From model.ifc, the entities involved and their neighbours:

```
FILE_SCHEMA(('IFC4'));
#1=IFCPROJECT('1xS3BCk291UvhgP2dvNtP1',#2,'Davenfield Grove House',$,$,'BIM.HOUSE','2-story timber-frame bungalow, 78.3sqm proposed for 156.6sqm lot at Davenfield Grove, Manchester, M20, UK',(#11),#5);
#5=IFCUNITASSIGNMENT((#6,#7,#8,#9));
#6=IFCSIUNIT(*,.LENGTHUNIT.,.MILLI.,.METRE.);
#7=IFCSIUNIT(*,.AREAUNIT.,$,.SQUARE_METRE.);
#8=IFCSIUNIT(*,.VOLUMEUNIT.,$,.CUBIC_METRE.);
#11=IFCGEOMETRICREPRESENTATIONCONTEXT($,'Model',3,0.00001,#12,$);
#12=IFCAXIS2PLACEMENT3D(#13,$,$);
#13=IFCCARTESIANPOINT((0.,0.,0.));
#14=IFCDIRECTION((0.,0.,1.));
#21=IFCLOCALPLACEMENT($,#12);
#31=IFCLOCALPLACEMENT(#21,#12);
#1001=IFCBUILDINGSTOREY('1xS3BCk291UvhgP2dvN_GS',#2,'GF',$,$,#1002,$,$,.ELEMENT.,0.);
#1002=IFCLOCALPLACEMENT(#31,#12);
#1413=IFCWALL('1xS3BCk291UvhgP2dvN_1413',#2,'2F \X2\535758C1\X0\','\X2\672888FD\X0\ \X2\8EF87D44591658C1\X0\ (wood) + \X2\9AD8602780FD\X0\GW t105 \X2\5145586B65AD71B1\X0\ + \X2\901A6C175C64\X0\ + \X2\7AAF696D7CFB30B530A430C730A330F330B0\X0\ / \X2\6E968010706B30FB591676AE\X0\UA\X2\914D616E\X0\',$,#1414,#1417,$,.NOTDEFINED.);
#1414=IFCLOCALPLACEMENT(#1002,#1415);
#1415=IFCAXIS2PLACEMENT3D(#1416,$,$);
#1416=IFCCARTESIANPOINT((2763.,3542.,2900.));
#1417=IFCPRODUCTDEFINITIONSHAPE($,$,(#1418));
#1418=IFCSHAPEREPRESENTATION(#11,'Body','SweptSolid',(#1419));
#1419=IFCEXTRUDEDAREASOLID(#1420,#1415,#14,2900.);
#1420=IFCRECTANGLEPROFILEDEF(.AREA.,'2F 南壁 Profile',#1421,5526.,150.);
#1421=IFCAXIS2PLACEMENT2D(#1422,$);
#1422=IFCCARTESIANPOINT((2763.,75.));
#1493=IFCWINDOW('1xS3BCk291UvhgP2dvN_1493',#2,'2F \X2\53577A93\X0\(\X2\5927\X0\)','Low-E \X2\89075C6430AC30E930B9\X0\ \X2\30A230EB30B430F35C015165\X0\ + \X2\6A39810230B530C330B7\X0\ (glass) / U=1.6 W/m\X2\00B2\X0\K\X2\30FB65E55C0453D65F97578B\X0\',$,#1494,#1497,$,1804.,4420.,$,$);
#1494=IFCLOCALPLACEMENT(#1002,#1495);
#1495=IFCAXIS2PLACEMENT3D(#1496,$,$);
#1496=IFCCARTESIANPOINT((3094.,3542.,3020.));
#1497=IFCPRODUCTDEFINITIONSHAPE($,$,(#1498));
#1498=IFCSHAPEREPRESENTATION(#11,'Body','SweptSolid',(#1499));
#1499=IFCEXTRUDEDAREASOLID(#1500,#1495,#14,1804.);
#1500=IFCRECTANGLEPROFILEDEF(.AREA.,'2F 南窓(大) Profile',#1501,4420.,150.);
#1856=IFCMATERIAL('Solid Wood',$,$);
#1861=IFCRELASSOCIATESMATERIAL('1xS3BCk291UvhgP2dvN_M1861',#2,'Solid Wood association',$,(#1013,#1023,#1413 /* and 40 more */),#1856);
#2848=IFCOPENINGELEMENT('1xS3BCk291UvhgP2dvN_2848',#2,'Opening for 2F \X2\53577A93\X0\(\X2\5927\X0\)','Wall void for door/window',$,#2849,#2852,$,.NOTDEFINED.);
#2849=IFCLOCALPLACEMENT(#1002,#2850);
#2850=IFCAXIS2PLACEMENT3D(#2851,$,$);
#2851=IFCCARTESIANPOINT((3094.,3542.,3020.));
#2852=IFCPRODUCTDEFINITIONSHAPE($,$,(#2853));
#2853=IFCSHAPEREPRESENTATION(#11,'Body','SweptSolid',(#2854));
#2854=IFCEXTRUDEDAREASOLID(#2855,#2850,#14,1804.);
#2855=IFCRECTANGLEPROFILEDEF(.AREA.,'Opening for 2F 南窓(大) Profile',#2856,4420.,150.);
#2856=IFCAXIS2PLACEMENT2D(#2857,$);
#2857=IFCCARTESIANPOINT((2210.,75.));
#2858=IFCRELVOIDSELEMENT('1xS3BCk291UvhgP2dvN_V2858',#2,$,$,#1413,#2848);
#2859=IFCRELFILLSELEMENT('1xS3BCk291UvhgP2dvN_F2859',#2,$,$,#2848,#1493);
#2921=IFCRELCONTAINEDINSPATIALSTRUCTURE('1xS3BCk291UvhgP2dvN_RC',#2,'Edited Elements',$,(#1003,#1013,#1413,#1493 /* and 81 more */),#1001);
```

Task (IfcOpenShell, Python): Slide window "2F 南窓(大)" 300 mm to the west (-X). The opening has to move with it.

```python
import ifcopenshell
import ifcopenshell.api.geometry
import ifcopenshell.util.placement

model = ifcopenshell.open("model.ifc")

window = model.by_guid("1xS3BCk291UvhgP2dvN_1493")
opening = window.FillsVoids[0].RelatingOpeningElement
wall = opening.VoidsElements[0].RelatingBuildingElement

wall_matrix = ifcopenshell.util.placement.get_local_placement(wall.ObjectPlacement)
shift = wall_matrix[:3, 0] * -300.0
before = ifcopenshell.util.placement.get_local_placement(window.ObjectPlacement)[:3, 3].copy()

# The window is not placed relative to its opening, so move both.
for product in (opening, window):
    matrix = ifcopenshell.util.placement.get_local_placement(product.ObjectPlacement)
    matrix[:3, 3] += shift
    ifcopenshell.api.geometry.edit_object_placement(model, product=product, matrix=matrix, is_si=False)

after = ifcopenshell.util.placement.get_local_placement(window.ObjectPlacement)[:3, 3]
print("window moved by", (after - before).round(3) + 0.0)

model.write("model_rev.ifc")
```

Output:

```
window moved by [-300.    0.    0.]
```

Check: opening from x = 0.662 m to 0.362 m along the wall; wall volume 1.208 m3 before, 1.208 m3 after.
